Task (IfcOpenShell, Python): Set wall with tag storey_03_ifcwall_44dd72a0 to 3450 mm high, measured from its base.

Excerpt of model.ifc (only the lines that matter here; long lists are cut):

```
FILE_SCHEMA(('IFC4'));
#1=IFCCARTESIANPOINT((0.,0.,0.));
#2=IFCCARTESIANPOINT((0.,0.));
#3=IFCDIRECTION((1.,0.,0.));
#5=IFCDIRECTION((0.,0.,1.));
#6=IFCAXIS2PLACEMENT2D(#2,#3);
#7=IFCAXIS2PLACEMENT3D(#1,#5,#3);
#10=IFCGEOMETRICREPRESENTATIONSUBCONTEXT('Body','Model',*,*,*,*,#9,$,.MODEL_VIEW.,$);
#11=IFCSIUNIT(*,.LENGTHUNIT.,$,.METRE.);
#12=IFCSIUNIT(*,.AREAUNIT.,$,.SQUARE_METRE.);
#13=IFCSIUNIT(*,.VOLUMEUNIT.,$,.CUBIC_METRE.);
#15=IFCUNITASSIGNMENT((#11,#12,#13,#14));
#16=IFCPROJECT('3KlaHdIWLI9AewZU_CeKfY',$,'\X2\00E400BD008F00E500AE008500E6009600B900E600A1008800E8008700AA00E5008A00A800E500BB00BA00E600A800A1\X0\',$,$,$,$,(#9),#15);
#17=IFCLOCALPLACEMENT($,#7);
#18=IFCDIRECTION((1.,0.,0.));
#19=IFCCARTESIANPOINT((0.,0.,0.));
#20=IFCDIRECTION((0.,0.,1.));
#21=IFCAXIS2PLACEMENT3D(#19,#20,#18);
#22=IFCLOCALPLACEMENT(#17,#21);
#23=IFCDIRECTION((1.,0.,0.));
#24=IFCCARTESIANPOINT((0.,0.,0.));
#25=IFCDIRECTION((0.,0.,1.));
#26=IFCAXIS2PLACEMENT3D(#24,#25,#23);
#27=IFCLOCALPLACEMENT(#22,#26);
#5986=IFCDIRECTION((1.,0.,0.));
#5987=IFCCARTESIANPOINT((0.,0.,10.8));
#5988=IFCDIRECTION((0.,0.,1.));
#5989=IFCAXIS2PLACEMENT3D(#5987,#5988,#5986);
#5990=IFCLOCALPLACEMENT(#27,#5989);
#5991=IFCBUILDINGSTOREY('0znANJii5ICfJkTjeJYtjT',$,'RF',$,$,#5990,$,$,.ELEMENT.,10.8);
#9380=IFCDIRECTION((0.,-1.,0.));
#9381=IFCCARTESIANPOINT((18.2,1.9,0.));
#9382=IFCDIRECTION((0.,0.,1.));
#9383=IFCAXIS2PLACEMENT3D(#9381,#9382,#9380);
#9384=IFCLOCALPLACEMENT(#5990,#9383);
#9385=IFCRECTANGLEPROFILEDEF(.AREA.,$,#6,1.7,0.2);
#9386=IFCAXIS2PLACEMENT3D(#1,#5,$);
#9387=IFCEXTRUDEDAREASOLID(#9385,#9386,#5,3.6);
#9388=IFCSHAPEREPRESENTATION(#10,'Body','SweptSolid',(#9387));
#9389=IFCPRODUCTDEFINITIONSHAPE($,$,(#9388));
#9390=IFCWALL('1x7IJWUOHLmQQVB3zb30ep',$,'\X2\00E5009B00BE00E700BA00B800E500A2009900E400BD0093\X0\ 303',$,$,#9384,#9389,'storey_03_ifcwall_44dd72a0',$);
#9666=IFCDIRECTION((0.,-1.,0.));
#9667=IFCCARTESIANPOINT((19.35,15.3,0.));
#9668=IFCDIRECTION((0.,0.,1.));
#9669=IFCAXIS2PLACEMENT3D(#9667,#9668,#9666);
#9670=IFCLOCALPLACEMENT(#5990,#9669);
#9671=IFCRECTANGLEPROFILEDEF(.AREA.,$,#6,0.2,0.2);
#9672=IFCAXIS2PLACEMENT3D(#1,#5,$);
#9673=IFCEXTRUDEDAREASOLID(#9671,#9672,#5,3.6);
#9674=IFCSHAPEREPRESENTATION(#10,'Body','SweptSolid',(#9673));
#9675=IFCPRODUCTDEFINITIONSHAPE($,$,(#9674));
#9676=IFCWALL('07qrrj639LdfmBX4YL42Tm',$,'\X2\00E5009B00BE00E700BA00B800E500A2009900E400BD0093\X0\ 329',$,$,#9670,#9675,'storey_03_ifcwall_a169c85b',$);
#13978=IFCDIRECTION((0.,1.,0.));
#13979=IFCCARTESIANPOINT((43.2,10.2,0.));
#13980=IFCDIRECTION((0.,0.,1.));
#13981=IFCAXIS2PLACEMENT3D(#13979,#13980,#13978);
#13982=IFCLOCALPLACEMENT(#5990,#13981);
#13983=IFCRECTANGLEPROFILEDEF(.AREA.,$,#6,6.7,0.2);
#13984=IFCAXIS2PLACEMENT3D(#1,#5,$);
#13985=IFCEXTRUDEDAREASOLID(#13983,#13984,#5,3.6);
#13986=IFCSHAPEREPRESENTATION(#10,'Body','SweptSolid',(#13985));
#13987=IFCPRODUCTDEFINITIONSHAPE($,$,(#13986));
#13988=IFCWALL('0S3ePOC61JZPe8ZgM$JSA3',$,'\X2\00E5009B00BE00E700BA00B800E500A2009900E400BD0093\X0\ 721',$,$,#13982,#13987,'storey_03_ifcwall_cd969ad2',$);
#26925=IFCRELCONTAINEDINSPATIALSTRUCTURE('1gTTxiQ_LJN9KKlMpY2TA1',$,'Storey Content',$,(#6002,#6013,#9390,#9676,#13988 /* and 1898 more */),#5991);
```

```python
import ifcopenshell
import ifcopenshell.geom
import ifcopenshell.util.representation
import ifcopenshell.util.shape
import ifcopenshell.util.unit

model = ifcopenshell.open("model.ifc")
unit_scale = ifcopenshell.util.unit.calculate_unit_scale(model)
settings = ifcopenshell.geom.settings()


def volume(element):
    """Net volume in cubic metres, openings subtracted."""
    shape = ifcopenshell.geom.create_shape(settings, element)
    return ifcopenshell.util.shape.get_volume(shape.geometry)


wall = model.by_guid("1x7IJWUOHLmQQVB3zb30ep")
before = volume(wall)

body = ifcopenshell.util.representation.get_representation(wall, "Model", "Body")
solid = body.Items[0]
old_height = solid.Depth
solid.Depth = 3.45 / unit_scale
after = volume(wall)

print(f"height {old_height:g} -> {solid.Depth:g}, volume {before:.3f} -> {after:.3f} m3")

model.write("model_v2.ifc")
```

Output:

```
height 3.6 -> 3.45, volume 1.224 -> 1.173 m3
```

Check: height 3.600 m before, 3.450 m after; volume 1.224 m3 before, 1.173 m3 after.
